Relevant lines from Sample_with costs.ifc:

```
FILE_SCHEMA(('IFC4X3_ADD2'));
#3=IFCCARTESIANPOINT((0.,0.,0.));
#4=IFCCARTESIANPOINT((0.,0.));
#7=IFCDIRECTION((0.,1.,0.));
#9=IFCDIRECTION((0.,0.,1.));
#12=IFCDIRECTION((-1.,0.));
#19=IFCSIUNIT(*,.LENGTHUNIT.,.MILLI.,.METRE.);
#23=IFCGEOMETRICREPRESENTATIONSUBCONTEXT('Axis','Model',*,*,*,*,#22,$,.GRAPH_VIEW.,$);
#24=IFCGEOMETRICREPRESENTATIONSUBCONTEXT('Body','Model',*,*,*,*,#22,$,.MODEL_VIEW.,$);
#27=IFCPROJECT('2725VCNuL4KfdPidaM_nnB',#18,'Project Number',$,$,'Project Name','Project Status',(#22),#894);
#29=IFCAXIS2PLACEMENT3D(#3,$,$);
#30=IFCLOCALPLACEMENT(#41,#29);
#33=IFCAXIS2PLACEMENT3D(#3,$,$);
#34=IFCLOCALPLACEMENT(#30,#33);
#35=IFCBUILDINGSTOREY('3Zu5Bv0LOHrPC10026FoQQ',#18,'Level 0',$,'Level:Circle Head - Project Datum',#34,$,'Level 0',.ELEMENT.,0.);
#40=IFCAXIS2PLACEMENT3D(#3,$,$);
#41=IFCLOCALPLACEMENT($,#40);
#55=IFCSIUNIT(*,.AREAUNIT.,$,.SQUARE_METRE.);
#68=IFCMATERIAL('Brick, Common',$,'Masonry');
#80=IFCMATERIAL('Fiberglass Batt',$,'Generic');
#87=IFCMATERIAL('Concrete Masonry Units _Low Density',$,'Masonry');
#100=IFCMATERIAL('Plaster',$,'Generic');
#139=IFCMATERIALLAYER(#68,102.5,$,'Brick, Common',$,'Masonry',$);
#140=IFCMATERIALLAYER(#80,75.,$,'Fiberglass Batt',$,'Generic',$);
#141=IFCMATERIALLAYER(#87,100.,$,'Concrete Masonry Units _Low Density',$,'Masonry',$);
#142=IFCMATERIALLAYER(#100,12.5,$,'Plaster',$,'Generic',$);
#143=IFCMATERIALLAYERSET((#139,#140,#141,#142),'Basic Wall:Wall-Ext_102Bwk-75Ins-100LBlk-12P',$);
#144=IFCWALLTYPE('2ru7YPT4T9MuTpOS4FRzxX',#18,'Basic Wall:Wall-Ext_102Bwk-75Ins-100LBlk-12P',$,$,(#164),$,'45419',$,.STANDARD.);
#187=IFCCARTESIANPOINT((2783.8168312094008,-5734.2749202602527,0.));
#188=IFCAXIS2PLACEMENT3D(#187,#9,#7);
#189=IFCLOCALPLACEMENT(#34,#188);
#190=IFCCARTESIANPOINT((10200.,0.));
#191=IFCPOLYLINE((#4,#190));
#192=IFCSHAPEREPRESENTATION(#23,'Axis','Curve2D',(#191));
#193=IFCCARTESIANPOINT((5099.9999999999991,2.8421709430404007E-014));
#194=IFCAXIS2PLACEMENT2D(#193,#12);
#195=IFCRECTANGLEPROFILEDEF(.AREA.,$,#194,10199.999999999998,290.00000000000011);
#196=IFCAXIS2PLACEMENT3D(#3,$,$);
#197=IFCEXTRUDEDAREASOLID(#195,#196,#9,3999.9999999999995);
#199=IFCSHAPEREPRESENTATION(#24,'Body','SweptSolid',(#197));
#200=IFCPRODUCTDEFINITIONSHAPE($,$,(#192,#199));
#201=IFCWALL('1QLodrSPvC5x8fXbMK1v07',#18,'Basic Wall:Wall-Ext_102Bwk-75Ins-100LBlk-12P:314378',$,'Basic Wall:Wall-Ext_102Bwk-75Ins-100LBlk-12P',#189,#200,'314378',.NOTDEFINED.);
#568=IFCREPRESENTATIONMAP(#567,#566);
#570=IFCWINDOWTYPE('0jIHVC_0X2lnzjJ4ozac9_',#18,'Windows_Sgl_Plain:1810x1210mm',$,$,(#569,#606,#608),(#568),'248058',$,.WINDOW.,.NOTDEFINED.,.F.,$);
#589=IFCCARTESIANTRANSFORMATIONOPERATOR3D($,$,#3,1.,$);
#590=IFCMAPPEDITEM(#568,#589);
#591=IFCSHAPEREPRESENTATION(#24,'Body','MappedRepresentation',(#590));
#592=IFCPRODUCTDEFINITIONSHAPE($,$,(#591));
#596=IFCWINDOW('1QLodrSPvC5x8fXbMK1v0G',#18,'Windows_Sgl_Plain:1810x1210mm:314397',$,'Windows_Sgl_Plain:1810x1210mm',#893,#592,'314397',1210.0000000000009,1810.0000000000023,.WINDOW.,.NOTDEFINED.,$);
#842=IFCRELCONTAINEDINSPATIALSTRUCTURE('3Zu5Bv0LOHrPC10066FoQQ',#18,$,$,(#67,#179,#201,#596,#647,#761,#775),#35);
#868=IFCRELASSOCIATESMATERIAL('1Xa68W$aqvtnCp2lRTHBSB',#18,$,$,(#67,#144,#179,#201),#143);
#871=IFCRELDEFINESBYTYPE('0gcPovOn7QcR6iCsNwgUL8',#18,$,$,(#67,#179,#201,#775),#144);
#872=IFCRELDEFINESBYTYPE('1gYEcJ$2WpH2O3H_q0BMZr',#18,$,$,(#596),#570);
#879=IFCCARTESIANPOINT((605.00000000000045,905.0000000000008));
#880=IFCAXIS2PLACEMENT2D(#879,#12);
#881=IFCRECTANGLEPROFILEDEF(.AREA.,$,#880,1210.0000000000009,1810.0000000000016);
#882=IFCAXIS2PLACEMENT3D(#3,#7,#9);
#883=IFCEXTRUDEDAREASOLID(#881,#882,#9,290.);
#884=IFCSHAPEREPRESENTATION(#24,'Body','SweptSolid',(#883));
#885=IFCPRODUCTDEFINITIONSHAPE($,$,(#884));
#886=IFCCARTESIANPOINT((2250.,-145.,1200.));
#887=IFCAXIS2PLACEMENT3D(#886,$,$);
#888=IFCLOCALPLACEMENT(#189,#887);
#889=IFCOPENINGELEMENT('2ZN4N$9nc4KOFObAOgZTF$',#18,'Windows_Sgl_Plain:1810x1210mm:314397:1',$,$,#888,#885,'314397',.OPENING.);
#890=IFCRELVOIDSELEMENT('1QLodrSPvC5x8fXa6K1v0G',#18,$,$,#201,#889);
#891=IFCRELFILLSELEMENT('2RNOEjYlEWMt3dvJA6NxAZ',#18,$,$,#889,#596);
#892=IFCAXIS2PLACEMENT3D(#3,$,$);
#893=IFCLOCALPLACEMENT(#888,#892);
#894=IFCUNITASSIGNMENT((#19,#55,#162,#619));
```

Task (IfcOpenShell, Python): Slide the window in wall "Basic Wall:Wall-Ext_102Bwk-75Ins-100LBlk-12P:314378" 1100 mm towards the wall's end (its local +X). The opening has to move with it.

```python
import ifcopenshell
import ifcopenshell.api.geometry
import ifcopenshell.util.placement
import ifcopenshell.util.unit

model = ifcopenshell.open("Sample_with costs.ifc")
unit_scale = ifcopenshell.util.unit.calculate_unit_scale(model)

window = model.by_guid("1QLodrSPvC5x8fXbMK1v0G")
opening = window.FillsVoids[0].RelatingOpeningElement
wall = opening.VoidsElements[0].RelatingBuildingElement

wall_matrix = ifcopenshell.util.placement.get_local_placement(wall.ObjectPlacement)
shift = wall_matrix[:3, 0] * 1.1 / unit_scale
before = ifcopenshell.util.placement.get_local_placement(window.ObjectPlacement)[:3, 3].copy()

# The window is placed relative to its opening, so it follows when the opening moves.
matrix = ifcopenshell.util.placement.get_local_placement(opening.ObjectPlacement)
matrix[:3, 3] += shift
ifcopenshell.api.geometry.edit_object_placement(
    model, product=opening, matrix=matrix, is_si=False, should_transform_children=True
)

after = ifcopenshell.util.placement.get_local_placement(window.ObjectPlacement)[:3, 3]
print("window moved by", (after - before).round(3) + 0.0)

model.write("Sample_with costs_edited.ifc")
```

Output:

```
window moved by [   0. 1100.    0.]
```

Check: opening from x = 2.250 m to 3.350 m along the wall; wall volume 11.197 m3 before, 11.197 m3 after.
